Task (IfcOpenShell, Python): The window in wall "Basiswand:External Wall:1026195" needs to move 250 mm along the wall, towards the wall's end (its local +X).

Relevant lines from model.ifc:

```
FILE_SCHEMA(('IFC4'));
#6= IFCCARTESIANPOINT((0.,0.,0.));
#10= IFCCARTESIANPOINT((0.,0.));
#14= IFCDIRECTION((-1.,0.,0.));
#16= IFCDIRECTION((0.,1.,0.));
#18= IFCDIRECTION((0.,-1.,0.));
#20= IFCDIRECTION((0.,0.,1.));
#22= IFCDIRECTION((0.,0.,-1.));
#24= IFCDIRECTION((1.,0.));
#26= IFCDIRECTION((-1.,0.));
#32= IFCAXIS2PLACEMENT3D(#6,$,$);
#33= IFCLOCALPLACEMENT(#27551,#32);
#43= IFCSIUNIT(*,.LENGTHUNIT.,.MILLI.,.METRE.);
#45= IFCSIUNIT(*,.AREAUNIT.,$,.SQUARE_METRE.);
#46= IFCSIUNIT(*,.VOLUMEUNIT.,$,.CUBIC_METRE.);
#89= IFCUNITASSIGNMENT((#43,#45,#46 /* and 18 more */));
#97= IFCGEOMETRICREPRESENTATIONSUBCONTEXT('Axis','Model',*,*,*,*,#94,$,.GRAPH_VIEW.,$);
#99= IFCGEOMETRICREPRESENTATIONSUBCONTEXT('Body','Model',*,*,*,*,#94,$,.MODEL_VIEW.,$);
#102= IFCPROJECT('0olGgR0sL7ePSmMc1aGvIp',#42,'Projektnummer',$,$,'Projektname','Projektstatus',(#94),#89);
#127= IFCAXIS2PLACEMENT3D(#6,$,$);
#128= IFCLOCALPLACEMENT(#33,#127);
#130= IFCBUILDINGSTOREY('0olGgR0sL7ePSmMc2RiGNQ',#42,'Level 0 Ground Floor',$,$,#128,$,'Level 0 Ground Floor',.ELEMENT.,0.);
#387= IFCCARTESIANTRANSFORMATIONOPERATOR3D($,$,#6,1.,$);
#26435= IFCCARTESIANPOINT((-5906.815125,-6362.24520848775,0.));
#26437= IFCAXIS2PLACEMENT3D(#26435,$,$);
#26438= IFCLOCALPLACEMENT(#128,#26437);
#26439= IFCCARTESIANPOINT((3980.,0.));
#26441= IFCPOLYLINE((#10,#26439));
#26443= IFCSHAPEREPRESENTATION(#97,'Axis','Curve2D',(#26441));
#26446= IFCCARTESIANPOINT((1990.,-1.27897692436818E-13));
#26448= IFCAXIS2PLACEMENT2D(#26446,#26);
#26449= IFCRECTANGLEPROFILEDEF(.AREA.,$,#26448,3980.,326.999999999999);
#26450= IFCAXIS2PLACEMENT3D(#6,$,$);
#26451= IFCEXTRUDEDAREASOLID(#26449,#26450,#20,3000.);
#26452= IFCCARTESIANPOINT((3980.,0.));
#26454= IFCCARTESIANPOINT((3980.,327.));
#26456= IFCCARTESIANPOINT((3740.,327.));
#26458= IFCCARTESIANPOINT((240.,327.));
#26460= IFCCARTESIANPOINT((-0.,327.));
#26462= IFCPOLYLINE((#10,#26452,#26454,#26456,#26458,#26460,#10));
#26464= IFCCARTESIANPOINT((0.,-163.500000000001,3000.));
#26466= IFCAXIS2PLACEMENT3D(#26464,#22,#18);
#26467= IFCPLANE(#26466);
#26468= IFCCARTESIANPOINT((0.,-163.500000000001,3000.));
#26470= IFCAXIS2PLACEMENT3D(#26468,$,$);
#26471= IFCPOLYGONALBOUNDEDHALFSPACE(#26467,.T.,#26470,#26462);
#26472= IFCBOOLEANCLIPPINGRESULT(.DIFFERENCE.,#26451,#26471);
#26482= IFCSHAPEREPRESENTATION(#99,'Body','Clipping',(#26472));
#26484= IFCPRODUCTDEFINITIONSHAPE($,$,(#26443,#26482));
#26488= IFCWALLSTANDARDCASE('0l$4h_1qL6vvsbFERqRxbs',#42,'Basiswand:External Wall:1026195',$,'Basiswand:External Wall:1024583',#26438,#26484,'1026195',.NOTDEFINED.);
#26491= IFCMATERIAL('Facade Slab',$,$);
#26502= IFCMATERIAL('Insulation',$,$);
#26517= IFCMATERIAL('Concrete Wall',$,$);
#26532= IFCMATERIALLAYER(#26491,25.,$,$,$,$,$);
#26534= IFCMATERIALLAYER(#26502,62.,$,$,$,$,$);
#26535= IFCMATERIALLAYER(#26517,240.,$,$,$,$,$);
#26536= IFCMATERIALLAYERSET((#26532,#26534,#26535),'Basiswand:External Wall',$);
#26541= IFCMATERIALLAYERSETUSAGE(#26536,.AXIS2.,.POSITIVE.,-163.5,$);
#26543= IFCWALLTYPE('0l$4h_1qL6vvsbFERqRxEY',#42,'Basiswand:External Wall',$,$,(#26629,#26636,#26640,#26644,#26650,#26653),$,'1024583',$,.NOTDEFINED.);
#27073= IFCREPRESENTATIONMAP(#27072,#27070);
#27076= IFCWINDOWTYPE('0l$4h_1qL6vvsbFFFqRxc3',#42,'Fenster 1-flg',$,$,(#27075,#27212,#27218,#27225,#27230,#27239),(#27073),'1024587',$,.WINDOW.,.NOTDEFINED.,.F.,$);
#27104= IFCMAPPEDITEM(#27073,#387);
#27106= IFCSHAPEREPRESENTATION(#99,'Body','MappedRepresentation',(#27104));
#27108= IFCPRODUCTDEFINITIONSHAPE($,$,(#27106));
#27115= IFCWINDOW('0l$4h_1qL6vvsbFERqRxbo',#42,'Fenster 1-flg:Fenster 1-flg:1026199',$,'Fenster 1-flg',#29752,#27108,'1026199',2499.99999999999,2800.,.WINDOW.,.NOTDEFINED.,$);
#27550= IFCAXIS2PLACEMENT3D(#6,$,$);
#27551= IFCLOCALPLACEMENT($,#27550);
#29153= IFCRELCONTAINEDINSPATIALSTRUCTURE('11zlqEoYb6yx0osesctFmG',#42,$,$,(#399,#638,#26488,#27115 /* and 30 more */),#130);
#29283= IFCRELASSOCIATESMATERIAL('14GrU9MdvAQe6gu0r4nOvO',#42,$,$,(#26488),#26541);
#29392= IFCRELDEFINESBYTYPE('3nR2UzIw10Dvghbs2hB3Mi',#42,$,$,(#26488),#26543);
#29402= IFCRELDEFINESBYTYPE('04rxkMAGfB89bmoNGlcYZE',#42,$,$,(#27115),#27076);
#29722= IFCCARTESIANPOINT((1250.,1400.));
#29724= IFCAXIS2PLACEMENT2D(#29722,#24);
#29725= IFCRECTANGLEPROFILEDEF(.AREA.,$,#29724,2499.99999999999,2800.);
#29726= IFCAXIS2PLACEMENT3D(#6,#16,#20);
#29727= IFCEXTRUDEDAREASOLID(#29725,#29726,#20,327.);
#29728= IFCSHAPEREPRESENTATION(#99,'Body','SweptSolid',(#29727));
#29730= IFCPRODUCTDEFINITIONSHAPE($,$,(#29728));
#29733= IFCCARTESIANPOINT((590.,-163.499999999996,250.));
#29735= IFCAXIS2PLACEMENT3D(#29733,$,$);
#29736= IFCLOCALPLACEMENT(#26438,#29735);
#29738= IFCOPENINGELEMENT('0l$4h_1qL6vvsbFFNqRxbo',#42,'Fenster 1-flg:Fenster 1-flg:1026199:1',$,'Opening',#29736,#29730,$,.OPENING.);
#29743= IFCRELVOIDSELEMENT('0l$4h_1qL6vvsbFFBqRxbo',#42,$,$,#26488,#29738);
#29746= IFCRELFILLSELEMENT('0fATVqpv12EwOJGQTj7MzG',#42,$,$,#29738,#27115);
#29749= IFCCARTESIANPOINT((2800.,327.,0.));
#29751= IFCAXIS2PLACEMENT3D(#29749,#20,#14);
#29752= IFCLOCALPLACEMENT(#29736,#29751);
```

```python
import ifcopenshell
import ifcopenshell.api.geometry
import ifcopenshell.util.placement
import ifcopenshell.util.unit

model = ifcopenshell.open("model.ifc")
unit_scale = ifcopenshell.util.unit.calculate_unit_scale(model)

window = model.by_guid("0l$4h_1qL6vvsbFERqRxbo")
opening = window.FillsVoids[0].RelatingOpeningElement
wall = opening.VoidsElements[0].RelatingBuildingElement

wall_matrix = ifcopenshell.util.placement.get_local_placement(wall.ObjectPlacement)
shift = wall_matrix[:3, 0] * 0.25 / unit_scale
before = ifcopenshell.util.placement.get_local_placement(window.ObjectPlacement)[:3, 3].copy()

# The window is placed relative to its opening, so it follows when the opening moves.
matrix = ifcopenshell.util.placement.get_local_placement(opening.ObjectPlacement)
matrix[:3, 3] += shift
ifcopenshell.api.geometry.edit_object_placement(
    model, product=opening, matrix=matrix, is_si=False, should_transform_children=True
)

after = ifcopenshell.util.placement.get_local_placement(window.ObjectPlacement)[:3, 3]
print("window moved by", (after - before).round(3) + 0.0)

model.write("model-out.ifc")
```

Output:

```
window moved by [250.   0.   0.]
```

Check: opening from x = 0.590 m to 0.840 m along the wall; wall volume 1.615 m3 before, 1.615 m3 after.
